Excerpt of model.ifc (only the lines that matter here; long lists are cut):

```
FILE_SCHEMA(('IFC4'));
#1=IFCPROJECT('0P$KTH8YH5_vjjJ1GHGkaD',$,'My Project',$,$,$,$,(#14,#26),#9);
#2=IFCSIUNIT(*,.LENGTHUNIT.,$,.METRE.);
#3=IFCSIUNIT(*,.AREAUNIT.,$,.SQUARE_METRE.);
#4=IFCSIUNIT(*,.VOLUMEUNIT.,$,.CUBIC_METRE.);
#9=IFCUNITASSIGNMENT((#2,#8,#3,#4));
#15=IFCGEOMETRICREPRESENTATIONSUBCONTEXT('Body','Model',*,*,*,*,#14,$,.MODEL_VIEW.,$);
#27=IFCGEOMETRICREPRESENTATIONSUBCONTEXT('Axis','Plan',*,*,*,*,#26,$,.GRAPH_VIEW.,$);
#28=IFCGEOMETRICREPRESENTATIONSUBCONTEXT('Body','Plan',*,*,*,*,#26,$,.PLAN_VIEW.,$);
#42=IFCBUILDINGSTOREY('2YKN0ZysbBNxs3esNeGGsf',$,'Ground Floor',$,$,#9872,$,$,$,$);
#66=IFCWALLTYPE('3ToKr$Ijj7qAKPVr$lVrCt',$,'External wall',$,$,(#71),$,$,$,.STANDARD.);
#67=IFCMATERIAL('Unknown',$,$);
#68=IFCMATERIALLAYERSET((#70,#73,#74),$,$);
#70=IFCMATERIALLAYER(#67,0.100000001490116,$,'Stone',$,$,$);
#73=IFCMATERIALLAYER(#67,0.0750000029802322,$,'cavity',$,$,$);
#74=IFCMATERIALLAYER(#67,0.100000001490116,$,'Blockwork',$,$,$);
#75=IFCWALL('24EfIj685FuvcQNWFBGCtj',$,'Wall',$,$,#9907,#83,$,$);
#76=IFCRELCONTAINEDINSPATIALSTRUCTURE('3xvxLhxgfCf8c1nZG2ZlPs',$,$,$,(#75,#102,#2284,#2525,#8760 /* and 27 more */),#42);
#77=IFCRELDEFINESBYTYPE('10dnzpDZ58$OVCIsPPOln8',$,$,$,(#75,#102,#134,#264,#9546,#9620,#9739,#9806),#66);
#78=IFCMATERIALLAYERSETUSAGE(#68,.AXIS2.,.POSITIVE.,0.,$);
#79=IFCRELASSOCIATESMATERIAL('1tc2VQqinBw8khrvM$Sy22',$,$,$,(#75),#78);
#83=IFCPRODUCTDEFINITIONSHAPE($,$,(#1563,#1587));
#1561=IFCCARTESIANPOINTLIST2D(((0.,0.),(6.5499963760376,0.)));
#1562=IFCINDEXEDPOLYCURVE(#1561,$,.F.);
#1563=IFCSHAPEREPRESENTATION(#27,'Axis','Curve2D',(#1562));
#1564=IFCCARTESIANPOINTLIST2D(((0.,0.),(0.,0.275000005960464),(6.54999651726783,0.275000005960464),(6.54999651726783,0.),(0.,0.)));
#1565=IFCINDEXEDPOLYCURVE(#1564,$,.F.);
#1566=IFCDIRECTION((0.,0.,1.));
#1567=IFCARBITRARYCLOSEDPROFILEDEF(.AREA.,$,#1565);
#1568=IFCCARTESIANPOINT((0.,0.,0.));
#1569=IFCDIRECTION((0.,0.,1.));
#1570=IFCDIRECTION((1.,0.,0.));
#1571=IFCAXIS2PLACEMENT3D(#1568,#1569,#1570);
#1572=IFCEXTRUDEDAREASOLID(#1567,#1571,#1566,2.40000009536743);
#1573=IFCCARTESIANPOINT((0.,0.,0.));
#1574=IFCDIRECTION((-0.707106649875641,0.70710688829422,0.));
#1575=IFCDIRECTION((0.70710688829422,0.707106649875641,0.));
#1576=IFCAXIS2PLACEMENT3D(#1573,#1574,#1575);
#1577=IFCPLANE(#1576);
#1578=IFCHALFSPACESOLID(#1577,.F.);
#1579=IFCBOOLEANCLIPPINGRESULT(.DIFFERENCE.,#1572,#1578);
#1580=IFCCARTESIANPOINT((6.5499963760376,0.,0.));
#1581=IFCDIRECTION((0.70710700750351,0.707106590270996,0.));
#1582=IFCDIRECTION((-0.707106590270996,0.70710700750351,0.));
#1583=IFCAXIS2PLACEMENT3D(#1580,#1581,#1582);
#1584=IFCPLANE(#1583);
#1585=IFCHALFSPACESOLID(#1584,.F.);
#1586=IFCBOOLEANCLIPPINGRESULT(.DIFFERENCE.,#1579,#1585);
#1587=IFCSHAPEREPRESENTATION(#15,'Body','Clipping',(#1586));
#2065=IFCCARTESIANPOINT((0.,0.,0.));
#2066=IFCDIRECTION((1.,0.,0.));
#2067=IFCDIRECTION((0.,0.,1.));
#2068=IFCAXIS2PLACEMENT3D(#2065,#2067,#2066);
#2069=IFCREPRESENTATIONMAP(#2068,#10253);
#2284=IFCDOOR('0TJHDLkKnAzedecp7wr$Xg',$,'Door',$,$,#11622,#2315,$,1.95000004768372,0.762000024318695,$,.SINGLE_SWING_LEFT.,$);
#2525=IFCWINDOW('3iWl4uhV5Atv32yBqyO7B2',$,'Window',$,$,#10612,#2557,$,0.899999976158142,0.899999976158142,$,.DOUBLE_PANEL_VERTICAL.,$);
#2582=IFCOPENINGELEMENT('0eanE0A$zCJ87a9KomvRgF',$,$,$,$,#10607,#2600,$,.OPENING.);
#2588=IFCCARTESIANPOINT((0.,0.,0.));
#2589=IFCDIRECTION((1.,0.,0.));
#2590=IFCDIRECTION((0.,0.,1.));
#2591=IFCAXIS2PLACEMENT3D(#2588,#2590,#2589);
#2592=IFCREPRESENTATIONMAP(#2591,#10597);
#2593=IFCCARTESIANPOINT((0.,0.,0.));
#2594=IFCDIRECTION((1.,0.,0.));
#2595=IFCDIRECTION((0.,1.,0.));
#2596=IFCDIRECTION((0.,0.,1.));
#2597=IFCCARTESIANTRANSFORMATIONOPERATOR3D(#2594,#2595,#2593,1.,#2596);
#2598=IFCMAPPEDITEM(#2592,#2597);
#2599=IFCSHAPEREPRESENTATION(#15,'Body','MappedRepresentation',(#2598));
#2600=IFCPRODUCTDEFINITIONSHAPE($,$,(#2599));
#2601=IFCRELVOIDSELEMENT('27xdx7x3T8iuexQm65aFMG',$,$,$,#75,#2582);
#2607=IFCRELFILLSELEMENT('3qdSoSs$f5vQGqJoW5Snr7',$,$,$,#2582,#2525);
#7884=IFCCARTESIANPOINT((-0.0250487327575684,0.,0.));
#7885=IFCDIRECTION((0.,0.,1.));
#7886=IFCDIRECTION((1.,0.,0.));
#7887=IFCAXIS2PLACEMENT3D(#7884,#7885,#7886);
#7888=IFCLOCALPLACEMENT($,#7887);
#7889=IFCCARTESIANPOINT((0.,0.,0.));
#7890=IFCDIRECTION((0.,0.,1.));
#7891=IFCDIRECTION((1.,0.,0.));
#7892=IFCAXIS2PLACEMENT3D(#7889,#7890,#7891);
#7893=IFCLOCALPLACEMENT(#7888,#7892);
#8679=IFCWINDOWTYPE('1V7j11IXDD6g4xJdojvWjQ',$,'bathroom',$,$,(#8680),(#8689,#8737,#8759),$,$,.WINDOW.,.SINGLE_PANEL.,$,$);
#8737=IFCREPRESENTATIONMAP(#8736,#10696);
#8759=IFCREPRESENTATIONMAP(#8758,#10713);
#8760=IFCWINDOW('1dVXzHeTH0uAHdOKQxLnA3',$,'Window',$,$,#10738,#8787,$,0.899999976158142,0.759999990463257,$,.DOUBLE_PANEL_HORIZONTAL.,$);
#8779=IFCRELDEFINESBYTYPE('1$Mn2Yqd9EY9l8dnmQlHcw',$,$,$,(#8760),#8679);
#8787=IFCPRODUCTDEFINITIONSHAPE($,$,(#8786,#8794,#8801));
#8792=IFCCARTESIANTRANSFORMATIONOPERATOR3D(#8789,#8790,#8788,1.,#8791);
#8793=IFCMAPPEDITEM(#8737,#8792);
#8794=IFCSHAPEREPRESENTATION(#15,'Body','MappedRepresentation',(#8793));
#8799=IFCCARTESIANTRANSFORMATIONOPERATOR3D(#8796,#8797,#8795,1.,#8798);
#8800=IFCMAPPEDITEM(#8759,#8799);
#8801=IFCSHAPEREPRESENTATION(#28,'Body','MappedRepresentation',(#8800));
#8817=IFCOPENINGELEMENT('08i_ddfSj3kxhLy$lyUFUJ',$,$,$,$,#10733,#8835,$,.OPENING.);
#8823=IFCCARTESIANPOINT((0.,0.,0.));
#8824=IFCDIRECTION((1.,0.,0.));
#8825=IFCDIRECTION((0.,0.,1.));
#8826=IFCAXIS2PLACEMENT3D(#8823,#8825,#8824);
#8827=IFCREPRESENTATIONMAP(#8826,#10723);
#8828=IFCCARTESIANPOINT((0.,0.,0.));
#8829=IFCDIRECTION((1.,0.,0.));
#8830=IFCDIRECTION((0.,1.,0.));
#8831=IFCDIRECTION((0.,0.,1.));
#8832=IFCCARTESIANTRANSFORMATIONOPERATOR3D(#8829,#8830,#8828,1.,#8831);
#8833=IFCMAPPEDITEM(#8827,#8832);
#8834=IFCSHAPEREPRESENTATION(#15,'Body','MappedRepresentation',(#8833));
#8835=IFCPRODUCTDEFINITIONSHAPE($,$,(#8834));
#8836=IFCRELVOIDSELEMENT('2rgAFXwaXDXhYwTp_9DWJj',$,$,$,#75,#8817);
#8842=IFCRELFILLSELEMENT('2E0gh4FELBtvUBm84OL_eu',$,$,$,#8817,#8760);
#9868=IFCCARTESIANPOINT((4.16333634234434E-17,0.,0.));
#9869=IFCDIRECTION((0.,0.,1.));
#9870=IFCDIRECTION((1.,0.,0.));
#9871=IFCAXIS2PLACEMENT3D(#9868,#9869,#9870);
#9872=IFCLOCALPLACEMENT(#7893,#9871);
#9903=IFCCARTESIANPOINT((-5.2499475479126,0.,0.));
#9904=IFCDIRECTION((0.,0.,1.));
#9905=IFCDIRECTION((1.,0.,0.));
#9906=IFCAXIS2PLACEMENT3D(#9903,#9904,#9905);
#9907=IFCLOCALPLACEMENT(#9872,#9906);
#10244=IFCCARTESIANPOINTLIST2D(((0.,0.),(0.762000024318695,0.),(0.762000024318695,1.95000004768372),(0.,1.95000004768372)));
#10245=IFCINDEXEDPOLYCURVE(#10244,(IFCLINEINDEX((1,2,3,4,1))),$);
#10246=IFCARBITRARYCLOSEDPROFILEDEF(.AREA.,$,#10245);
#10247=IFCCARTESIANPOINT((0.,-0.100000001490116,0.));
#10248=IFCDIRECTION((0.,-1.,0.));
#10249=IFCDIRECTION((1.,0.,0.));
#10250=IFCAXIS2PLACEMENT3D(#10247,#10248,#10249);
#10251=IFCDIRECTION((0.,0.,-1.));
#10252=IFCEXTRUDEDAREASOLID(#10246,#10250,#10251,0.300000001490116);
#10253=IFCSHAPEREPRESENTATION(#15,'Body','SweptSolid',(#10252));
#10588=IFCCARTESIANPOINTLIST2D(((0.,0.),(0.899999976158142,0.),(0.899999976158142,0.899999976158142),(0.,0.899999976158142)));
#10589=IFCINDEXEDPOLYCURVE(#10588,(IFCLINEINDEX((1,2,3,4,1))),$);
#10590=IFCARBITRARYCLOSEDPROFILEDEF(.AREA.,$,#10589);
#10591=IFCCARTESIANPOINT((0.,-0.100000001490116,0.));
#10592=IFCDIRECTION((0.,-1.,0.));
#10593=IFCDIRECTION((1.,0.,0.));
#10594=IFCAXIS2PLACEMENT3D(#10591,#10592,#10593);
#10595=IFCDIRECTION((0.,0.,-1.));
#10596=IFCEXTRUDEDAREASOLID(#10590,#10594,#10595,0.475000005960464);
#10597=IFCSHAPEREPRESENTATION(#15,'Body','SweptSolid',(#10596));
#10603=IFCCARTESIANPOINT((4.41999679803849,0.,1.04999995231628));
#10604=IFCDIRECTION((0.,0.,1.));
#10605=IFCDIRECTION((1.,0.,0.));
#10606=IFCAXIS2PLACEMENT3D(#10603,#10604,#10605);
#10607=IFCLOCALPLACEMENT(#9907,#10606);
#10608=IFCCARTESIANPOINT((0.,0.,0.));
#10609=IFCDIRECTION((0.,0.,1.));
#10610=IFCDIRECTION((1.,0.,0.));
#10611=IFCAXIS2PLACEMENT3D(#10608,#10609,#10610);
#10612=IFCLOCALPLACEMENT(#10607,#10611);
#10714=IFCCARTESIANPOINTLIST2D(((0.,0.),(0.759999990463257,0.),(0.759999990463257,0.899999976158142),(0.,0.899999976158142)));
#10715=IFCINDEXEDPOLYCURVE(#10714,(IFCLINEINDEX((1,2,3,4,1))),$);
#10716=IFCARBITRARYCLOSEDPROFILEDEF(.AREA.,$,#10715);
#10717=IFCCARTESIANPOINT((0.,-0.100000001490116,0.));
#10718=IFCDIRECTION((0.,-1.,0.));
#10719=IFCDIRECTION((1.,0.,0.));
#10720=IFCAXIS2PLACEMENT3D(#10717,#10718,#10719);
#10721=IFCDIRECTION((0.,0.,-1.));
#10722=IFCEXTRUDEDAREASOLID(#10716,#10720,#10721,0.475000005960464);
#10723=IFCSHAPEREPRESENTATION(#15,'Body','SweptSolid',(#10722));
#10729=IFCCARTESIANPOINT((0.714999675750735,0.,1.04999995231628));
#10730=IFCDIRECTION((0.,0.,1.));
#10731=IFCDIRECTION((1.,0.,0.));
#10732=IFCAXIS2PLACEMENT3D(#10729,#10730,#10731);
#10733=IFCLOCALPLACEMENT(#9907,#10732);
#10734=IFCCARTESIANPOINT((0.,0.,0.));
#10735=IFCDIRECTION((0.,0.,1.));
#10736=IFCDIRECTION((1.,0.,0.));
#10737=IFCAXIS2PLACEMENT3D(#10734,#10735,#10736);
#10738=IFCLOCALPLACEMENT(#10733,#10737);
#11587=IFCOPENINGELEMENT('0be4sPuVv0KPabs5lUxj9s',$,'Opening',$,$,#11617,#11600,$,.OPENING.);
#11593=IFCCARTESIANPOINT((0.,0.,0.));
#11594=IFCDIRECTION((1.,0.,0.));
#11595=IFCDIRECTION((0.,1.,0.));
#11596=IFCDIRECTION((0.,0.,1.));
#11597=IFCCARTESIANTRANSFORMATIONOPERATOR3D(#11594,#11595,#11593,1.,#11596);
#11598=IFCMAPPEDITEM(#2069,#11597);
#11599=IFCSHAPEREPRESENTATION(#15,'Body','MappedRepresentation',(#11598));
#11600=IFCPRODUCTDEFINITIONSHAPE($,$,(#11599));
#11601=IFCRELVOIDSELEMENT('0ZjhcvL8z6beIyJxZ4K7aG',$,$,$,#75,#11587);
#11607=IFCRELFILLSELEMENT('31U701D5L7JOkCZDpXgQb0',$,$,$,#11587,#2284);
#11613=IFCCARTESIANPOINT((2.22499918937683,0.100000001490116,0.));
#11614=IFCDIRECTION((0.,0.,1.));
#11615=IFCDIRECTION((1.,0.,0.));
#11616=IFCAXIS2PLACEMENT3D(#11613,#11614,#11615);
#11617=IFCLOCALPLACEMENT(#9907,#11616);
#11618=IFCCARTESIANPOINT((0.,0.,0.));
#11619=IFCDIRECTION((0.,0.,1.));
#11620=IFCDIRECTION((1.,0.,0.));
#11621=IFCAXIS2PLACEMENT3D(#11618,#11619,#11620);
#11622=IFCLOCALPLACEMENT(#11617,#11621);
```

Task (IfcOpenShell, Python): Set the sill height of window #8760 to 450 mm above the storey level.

```python
import numpy as np
import ifcopenshell
import ifcopenshell.api.geometry
import ifcopenshell.geom
import ifcopenshell.util.element
import ifcopenshell.util.placement
import ifcopenshell.util.shape
import ifcopenshell.util.unit

model = ifcopenshell.open("model.ifc")
unit_scale = ifcopenshell.util.unit.calculate_unit_scale(model)

window = model.by_id(8760)
opening = window.FillsVoids[0].RelatingOpeningElement
storey = ifcopenshell.util.element.get_container(window, ifc_class="IfcBuildingStorey")
level = ifcopenshell.util.placement.get_local_placement(storey.ObjectPlacement)[2, 3]

# The opening's origin need not be at the sill, so measure its lowest point.
shape = ifcopenshell.geom.create_shape(ifcopenshell.geom.settings(), opening)
bottom = ifcopenshell.util.shape.get_shape_bottom_elevation(shape, shape.geometry) / unit_scale
dz = level + 0.45 - bottom

shift = np.array([0.0, 0.0, dz])
# The window is placed relative to its opening, so it follows when the opening moves.
matrix = ifcopenshell.util.placement.get_local_placement(opening.ObjectPlacement)
matrix[:3, 3] += shift
ifcopenshell.api.geometry.edit_object_placement(
    model, product=opening, matrix=matrix, is_si=False, should_transform_children=True
)

print(f"moved by {dz * unit_scale:+.3f} m")

model.write("model_rev.ifc")
```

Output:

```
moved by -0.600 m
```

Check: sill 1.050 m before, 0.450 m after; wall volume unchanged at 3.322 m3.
